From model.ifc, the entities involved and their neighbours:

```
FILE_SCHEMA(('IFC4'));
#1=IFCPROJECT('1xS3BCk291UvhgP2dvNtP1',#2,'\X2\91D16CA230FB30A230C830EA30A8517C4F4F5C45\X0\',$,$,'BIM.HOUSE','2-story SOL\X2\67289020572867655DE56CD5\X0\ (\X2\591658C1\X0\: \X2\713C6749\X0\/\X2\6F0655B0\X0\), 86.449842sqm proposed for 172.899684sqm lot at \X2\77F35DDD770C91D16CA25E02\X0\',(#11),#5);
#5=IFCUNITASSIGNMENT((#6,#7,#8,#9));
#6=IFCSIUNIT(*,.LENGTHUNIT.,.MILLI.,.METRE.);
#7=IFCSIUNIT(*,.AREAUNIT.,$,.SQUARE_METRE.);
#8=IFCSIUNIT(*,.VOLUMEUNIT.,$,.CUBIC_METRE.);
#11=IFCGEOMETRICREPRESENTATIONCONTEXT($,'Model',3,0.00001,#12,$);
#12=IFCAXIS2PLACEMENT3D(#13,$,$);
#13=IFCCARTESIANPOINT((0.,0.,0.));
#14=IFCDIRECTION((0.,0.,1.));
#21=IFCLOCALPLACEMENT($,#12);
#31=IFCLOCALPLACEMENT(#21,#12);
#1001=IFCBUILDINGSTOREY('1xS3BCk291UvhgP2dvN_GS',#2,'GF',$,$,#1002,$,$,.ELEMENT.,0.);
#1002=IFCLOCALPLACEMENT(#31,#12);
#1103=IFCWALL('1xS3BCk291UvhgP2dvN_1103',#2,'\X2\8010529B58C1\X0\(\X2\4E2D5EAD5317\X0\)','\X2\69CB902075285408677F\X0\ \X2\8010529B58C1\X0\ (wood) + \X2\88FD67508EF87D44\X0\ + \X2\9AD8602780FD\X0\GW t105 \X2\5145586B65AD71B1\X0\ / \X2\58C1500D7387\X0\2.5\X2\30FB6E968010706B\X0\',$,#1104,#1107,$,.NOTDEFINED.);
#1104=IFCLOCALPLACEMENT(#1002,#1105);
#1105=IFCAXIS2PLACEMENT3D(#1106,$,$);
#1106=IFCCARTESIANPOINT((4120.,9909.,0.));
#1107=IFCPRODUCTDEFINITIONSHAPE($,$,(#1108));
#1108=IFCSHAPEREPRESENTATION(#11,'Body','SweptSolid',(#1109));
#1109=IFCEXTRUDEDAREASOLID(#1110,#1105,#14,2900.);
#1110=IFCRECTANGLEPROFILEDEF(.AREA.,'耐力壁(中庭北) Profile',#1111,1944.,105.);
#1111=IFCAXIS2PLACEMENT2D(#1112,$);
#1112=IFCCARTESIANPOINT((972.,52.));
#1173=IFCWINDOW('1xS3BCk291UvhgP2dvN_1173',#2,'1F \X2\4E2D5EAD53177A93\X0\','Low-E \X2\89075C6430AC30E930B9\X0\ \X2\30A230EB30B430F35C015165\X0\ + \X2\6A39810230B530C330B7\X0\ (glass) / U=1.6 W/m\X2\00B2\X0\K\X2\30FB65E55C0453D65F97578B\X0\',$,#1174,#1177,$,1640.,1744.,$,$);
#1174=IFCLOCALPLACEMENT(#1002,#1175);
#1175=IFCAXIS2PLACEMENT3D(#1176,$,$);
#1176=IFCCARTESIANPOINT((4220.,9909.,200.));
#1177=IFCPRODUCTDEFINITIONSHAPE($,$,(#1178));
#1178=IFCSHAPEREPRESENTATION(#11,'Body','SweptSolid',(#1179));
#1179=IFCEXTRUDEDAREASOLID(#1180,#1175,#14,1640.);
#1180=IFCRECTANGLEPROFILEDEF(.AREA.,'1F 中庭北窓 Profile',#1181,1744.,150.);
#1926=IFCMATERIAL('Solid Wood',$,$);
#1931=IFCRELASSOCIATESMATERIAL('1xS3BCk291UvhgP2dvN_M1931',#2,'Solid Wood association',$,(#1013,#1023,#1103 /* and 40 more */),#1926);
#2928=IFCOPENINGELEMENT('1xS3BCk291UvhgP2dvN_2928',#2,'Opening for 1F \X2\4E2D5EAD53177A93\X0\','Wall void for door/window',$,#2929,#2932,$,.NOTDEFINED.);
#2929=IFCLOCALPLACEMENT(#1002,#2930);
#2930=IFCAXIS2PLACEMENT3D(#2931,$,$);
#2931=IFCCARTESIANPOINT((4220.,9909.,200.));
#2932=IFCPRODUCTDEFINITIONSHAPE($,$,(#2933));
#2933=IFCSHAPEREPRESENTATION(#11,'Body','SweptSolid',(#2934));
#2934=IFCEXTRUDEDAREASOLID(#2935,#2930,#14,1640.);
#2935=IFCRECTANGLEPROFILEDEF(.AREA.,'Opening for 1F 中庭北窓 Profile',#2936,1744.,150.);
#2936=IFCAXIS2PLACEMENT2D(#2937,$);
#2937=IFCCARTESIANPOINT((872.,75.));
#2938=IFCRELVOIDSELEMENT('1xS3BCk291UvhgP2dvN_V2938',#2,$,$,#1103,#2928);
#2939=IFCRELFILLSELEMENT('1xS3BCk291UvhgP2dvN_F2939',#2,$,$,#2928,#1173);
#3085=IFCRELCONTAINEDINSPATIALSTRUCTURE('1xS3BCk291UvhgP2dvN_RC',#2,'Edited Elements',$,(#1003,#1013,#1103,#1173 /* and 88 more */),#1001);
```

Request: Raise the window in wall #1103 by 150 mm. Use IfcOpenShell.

```python
import numpy as np
import ifcopenshell
import ifcopenshell.api.geometry
import ifcopenshell.util.placement
import ifcopenshell.util.unit

model = ifcopenshell.open("model.ifc")
unit_scale = ifcopenshell.util.unit.calculate_unit_scale(model)

window = model.by_id(1173)
opening = window.FillsVoids[0].RelatingOpeningElement
dz = 150.0

shift = np.array([0.0, 0.0, dz])
# The window is not placed relative to its opening, so move both.
for product in (opening, window):
    matrix = ifcopenshell.util.placement.get_local_placement(product.ObjectPlacement)
    matrix[:3, 3] += shift
    ifcopenshell.api.geometry.edit_object_placement(model, product=product, matrix=matrix, is_si=False)

print(f"moved by {dz * unit_scale:+.3f} m")

model.write("model-out.ifc")
```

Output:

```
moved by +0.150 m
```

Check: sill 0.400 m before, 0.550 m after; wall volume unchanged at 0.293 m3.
